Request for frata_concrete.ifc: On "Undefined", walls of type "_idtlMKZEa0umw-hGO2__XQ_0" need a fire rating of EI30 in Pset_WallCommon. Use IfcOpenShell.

First a look at what the model holds.

```python
import ifcopenshell
import ifcopenshell.util.element

model = ifcopenshell.open("frata_concrete.ifc")
print(model.schema)
storey = next(s for s in model.by_type("IfcBuildingStorey") if s.Name == "Undefined")
walls = [e for e in ifcopenshell.util.element.get_decomposition(storey) if e.is_a("IfcWall")]
seen = {}
for e in walls:
    element_type = ifcopenshell.util.element.get_type(e)
    key = (element_type.Name if element_type != e and element_type else None, ifcopenshell.util.element.get_pset(e, "Pset_WallCommon", "FireRating"))
    seen[key] = seen.get(key, 0) + 1
for (name, value), count in sorted(seen.items(), key=str):
    print(count, "x", name, "|", value)
```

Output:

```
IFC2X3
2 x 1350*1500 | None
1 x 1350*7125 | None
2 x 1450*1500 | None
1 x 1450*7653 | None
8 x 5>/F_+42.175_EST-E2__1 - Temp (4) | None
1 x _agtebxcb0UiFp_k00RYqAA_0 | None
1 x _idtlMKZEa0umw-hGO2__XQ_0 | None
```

```python
import ifcopenshell
import ifcopenshell.api.pset
import ifcopenshell.util.element

model = ifcopenshell.open("frata_concrete.ifc")

storey = next(s for s in model.by_type("IfcBuildingStorey") if s.Name == "Undefined")
walls = [e for e in ifcopenshell.util.element.get_decomposition(storey) if e.is_a("IfcWall")]

count = 0
for e in walls:
    element_type = ifcopenshell.util.element.get_type(e)
    if element_type in (None, e) or element_type.Name != "_idtlMKZEa0umw-hGO2__XQ_0":
        continue
    # add_pset returns the element's existing set when there is one.
    pset = ifcopenshell.api.pset.add_pset(model, product=e, name="Pset_WallCommon")
    ifcopenshell.api.pset.edit_pset(model, pset=pset, properties={"FireRating": "EI30"})
    count += 1

print(count, "walls updated")

model.write("frata_concrete_rev.ifc")
```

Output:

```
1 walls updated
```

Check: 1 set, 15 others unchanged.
